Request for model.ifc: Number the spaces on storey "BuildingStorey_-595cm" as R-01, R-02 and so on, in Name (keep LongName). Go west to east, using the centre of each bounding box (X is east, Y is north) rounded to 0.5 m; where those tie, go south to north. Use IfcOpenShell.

First a look at what the model holds.

```python
import ifcopenshell
import ifcopenshell.util.element
import ifcopenshell.util.placement

model = ifcopenshell.open("model.ifc")
print(model.schema)
storey = next(s for s in model.by_type("IfcBuildingStorey") if s.Name == "BuildingStorey_-595cm")
spaces = [e for e in ifcopenshell.util.element.get_decomposition(storey) if e.is_a("IfcSpace")]
for e in sorted(spaces, key=lambda e: e.id()):
    origin = ifcopenshell.util.placement.get_local_placement(e.ObjectPlacement)[:3, 3]
    print(e.id(), e.Name, e.LongName, origin.round(2) + 0.0, sep=" | ")
```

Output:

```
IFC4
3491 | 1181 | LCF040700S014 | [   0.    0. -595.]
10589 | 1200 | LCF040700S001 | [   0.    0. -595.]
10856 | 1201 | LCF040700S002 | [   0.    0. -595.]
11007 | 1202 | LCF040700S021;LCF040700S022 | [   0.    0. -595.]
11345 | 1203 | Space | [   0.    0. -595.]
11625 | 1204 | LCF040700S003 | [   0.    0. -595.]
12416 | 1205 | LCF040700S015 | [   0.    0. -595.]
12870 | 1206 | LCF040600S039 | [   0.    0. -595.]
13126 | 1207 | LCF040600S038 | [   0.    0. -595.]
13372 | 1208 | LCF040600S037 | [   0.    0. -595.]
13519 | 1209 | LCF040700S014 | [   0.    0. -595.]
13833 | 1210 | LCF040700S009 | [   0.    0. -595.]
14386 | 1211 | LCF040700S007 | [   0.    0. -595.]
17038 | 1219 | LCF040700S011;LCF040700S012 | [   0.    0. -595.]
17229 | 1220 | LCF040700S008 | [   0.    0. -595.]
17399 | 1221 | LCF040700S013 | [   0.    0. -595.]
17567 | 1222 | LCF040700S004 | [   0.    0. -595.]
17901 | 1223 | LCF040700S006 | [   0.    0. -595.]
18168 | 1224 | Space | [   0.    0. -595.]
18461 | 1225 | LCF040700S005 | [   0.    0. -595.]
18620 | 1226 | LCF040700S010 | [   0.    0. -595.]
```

```python
import ifcopenshell
import ifcopenshell.geom
import ifcopenshell.util.element
import ifcopenshell.util.shape

model = ifcopenshell.open("model.ifc")
settings = ifcopenshell.geom.settings()
settings.set("use-world-coords", True)


def centre(element):
    shape = ifcopenshell.geom.create_shape(settings, element)
    return ifcopenshell.util.shape.get_bbox_centroid(shape.geometry)


storey = next(s for s in model.by_type("IfcBuildingStorey") if s.Name == "BuildingStorey_-595cm")
spaces = [e for e in ifcopenshell.util.element.get_decomposition(storey) if e.is_a("IfcSpace")]

# Insertion points can sit at a corner or the storey origin, so sort by the geometry (in metres).
centres = {e: centre(e) for e in spaces}
spaces.sort(key=lambda e: (round(centres[e][0] / 0.5), centres[e][1]))

for i, e in enumerate(spaces, start=1):
    number = f"R-{i:02d}"
    e.Name = number
    print(e.id(), number)

model.write("model-out.ifc")
```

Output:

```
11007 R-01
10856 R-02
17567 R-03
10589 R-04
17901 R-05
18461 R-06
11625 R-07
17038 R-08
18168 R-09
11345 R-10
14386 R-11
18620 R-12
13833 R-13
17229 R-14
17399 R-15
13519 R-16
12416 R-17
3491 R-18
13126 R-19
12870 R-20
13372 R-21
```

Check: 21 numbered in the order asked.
